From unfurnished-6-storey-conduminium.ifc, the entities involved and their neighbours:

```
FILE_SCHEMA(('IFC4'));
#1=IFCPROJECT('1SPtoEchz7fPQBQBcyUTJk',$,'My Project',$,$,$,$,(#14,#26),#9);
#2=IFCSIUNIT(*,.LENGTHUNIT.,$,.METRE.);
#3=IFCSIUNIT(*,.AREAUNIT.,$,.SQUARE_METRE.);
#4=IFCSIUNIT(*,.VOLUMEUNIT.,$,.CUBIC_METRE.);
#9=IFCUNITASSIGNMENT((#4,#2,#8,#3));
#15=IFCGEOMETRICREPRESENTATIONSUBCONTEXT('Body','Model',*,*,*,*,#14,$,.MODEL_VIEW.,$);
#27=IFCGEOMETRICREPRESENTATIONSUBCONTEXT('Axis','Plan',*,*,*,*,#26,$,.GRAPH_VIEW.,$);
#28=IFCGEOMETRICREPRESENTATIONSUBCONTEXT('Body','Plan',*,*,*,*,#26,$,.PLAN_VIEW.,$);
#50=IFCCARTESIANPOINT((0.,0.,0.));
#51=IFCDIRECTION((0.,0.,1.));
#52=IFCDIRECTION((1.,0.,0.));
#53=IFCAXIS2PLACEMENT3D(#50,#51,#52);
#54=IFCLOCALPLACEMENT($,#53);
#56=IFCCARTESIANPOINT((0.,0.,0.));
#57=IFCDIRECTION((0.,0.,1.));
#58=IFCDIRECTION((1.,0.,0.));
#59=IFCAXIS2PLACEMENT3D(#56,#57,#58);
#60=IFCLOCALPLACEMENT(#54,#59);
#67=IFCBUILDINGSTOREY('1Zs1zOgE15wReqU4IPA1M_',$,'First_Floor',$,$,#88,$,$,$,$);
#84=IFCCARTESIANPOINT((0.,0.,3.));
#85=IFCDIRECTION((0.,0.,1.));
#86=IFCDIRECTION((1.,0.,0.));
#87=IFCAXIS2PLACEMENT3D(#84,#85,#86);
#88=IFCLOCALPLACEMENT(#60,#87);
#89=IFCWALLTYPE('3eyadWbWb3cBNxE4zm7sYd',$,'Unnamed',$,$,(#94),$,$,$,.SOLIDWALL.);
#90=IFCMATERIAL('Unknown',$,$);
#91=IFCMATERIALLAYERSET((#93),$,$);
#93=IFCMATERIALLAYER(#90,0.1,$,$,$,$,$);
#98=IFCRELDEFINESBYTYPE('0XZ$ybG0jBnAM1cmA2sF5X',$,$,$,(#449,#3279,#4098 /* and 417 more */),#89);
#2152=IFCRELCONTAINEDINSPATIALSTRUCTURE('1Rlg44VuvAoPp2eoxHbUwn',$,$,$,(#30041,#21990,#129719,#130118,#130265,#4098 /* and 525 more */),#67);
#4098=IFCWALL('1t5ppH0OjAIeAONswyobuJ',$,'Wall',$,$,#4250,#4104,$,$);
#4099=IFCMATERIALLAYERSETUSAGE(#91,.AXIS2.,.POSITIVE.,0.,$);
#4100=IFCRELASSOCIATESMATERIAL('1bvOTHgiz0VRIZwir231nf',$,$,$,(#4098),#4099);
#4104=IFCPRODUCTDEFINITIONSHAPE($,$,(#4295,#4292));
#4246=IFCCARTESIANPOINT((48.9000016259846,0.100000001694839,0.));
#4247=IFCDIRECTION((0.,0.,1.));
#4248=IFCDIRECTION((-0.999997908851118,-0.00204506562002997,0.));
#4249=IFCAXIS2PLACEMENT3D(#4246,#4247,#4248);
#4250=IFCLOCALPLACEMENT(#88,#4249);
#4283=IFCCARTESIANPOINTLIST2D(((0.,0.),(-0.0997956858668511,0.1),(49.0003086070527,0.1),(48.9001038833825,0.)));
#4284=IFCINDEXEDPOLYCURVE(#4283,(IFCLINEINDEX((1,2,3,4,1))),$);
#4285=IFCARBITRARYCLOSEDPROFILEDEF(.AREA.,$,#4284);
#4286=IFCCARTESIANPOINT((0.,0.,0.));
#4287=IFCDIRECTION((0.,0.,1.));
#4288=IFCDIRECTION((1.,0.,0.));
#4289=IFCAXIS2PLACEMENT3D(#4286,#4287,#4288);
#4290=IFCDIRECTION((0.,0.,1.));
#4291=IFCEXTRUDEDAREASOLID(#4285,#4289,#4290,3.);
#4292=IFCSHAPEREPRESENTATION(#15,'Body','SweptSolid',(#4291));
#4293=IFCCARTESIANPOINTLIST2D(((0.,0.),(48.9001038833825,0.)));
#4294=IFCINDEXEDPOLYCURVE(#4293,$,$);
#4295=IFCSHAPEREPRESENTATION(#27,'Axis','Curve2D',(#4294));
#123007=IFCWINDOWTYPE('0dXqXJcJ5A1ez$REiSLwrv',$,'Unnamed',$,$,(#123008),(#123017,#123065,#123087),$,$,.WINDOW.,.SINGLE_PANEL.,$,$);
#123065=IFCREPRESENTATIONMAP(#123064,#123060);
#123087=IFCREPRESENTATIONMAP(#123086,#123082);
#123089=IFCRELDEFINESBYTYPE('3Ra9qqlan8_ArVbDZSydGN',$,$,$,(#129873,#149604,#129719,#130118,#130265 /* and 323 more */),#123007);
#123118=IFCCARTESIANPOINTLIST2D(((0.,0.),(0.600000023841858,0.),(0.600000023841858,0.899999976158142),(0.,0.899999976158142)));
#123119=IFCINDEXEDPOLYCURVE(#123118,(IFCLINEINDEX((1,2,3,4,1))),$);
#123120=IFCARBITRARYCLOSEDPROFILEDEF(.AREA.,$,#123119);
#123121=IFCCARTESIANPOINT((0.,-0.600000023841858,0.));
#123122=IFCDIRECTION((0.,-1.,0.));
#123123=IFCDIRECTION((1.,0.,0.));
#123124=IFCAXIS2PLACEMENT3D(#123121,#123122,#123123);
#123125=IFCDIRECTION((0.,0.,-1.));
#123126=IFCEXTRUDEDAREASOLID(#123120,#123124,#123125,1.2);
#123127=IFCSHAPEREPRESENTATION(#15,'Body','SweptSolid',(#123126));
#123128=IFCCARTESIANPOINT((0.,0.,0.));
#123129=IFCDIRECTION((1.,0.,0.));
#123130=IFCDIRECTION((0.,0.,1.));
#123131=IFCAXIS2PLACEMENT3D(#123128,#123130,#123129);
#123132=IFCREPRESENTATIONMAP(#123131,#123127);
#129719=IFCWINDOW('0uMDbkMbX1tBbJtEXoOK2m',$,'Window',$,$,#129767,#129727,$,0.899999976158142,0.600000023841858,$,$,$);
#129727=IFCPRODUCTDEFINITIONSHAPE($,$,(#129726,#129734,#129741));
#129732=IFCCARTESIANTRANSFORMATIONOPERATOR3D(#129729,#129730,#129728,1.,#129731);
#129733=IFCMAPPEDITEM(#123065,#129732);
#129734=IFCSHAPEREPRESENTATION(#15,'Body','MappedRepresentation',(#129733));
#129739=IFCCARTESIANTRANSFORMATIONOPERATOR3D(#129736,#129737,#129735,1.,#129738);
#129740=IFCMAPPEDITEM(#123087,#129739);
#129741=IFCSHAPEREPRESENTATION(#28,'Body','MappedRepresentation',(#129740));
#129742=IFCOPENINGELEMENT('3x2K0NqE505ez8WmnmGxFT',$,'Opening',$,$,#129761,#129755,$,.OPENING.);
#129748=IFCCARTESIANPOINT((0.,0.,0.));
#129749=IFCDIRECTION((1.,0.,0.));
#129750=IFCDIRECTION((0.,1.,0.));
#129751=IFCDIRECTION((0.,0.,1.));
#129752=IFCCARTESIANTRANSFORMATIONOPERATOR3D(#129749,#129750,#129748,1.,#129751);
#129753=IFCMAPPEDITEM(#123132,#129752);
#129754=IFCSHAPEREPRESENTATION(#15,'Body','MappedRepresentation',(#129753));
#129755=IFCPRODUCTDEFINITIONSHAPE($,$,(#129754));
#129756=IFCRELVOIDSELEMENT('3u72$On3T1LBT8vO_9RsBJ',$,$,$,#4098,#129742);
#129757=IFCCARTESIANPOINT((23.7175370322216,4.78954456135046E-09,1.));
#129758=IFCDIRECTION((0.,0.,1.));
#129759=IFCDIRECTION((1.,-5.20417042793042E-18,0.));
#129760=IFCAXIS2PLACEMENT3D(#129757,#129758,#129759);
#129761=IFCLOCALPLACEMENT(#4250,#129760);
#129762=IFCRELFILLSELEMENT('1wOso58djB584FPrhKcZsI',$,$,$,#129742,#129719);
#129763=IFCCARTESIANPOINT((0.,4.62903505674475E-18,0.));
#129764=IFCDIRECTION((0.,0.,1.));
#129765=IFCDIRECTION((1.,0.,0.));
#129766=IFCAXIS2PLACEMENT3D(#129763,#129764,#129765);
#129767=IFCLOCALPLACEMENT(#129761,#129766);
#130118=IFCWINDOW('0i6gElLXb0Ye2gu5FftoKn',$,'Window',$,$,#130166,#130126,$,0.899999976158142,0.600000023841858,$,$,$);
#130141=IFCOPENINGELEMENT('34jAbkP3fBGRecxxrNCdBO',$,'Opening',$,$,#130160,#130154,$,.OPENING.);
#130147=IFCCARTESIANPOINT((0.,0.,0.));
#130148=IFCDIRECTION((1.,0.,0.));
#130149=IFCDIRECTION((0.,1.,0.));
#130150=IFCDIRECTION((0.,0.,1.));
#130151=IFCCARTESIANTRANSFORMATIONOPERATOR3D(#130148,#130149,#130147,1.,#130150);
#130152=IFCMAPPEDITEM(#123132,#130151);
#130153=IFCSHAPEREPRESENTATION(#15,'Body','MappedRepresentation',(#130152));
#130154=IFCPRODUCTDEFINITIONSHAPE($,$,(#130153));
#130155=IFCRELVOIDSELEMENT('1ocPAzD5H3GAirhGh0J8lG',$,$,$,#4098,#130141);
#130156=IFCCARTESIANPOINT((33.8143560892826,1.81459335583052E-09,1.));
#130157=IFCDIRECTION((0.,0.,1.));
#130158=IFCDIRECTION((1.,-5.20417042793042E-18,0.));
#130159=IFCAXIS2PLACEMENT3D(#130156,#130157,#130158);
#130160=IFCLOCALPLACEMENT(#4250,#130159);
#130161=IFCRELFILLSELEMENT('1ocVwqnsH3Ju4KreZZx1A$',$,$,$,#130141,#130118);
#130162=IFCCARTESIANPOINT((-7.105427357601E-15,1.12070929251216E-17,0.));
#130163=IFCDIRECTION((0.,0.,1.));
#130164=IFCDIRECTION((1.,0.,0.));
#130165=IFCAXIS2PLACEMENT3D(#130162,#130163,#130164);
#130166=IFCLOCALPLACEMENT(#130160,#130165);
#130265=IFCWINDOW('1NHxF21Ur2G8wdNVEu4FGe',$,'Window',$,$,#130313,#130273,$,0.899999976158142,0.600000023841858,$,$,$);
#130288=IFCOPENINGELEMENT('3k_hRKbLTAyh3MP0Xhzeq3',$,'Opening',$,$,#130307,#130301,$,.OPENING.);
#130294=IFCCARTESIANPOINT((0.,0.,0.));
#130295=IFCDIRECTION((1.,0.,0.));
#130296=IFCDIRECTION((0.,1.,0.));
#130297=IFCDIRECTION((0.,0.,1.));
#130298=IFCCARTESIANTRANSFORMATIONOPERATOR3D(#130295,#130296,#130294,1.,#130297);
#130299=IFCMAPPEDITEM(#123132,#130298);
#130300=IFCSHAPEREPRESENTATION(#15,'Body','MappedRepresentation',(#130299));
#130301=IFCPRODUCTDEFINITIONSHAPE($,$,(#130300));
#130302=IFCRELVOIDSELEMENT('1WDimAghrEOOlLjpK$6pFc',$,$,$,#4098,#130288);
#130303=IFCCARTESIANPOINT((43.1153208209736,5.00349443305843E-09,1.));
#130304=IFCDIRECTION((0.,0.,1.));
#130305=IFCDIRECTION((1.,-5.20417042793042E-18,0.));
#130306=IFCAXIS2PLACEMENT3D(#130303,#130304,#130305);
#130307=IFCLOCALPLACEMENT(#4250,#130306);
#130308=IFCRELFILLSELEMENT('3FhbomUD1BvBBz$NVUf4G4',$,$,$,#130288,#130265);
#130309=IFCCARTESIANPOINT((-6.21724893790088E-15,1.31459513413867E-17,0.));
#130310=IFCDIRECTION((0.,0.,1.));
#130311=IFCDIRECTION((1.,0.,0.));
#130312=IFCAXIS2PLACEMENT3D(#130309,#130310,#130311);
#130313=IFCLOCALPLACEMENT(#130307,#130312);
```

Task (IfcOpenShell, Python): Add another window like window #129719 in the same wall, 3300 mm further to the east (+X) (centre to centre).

```python
import ifcopenshell
import ifcopenshell.api.feature
import ifcopenshell.api.geometry
import ifcopenshell.api.root
import ifcopenshell.geom
import ifcopenshell.util.element
import ifcopenshell.util.placement
import ifcopenshell.util.shape

model = ifcopenshell.open("unfurnished-6-storey-conduminium.ifc")
settings = ifcopenshell.geom.settings()


def volume(element):
    """Net volume in cubic metres, openings subtracted."""
    shape = ifcopenshell.geom.create_shape(settings, element)
    return ifcopenshell.util.shape.get_volume(shape.geometry)


window = model.by_guid("0uMDbkMbX1tBbJtEXoOK2m")
opening = window.FillsVoids[0].RelatingOpeningElement
wall = opening.VoidsElements[0].RelatingBuildingElement
before = volume(wall)
shift = ifcopenshell.util.placement.get_local_placement(wall.ObjectPlacement)[:3, 0] * -3.3

# copy_class copies the void relationship, type, container and properties, but no geometry.
new_opening = ifcopenshell.api.root.copy_class(model, product=opening)
new_opening.Representation = ifcopenshell.util.element.copy_deep(
    model, opening.Representation, exclude=["IfcGeometricRepresentationContext", "IfcRepresentationMap"]
)
new_window = ifcopenshell.api.root.copy_class(model, product=window)
new_window.Representation = ifcopenshell.util.element.copy_deep(
    model, window.Representation, exclude=["IfcGeometricRepresentationContext", "IfcRepresentationMap"]
)
ifcopenshell.api.feature.add_filling(model, opening=new_opening, element=new_window)

for old, new in ((opening, new_opening), (window, new_window)):
    matrix = ifcopenshell.util.placement.get_local_placement(old.ObjectPlacement)
    matrix[:3, 3] += shift
    ifcopenshell.api.geometry.edit_object_placement(model, product=new, matrix=matrix, is_si=False)

after = volume(wall)

print(f"wall volume {before:.3f} -> {after:.3f} m3")

model.write("unfurnished-6-storey-conduminium_edited.ifc")
```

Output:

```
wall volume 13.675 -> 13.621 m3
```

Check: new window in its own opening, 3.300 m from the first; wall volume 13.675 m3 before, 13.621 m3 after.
